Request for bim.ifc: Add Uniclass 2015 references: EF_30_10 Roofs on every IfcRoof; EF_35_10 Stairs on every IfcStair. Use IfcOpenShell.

First a look at what the model holds.

```python
import ifcopenshell

model = ifcopenshell.open("bim.ifc")
print(model.schema)
print("classifications:", [c.Name for c in model.by_type("IfcClassification")])
for ifc_class in ("IfcDoor", "IfcRoof", "IfcStair", "IfcWall", "IfcWindow"):
    print(ifc_class, len(model.by_type(ifc_class)))
```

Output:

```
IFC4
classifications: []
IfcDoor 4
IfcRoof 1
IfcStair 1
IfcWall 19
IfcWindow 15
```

```python
import ifcopenshell
import ifcopenshell.api.classification

model = ifcopenshell.open("bim.ifc")

system = ifcopenshell.api.classification.add_classification(model, classification="Uniclass 2015")

codes = {
    "IfcRoof": ("EF_30_10", "Roofs"),
    "IfcStair": ("EF_35_10", "Stairs"),
}
for ifc_class, (code, name) in codes.items():
    products = model.by_type(ifc_class)
    ifcopenshell.api.classification.add_reference(
        model, products=products, classification=system, identification=code, name=name
    )
    print(code, len(products))

model.write("bim_updated.ifc")
```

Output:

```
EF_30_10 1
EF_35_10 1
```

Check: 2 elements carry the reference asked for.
